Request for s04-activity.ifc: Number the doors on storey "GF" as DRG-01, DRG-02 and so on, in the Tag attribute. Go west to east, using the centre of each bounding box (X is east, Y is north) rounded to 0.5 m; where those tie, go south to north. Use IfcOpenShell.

First a look at what the model holds.

```python
import ifcopenshell
import ifcopenshell.util.element
import ifcopenshell.util.placement

model = ifcopenshell.open("s04-activity.ifc")
print(model.schema)
storey = next(s for s in model.by_type("IfcBuildingStorey") if s.Name == "GF")
doors = [e for e in ifcopenshell.util.element.get_decomposition(storey) if e.is_a("IfcDoor")]
for e in sorted(doors, key=lambda e: e.id()):
    origin = ifcopenshell.util.placement.get_local_placement(e.ObjectPlacement)[:3, 3]
    print(e.id(), e.Tag, e.Name, origin.round(2) + 0.0, sep=" | ")
```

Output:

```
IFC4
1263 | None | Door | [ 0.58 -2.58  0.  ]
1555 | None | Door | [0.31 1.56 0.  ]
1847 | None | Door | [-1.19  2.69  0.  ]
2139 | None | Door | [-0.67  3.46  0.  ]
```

```python
import ifcopenshell
import ifcopenshell.geom
import ifcopenshell.util.element
import ifcopenshell.util.shape

model = ifcopenshell.open("s04-activity.ifc")
settings = ifcopenshell.geom.settings()
settings.set("use-world-coords", True)


def centre(element):
    shape = ifcopenshell.geom.create_shape(settings, element)
    return ifcopenshell.util.shape.get_bbox_centroid(shape.geometry)


storey = next(s for s in model.by_type("IfcBuildingStorey") if s.Name == "GF")
doors = [e for e in ifcopenshell.util.element.get_decomposition(storey) if e.is_a("IfcDoor")]

# Insertion points can sit at a corner or the storey origin, so sort by the geometry (in metres).
centres = {e: centre(e) for e in doors}
doors.sort(key=lambda e: (round(centres[e][0] / 0.5), centres[e][1]))

for i, e in enumerate(doors, start=1):
    number = f"DRG-{i:02d}"
    e.Tag = number
    print(e.id(), number)

model.write("s04-activity-out.ifc")
```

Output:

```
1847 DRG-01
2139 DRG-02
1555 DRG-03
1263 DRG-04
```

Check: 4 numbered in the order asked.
